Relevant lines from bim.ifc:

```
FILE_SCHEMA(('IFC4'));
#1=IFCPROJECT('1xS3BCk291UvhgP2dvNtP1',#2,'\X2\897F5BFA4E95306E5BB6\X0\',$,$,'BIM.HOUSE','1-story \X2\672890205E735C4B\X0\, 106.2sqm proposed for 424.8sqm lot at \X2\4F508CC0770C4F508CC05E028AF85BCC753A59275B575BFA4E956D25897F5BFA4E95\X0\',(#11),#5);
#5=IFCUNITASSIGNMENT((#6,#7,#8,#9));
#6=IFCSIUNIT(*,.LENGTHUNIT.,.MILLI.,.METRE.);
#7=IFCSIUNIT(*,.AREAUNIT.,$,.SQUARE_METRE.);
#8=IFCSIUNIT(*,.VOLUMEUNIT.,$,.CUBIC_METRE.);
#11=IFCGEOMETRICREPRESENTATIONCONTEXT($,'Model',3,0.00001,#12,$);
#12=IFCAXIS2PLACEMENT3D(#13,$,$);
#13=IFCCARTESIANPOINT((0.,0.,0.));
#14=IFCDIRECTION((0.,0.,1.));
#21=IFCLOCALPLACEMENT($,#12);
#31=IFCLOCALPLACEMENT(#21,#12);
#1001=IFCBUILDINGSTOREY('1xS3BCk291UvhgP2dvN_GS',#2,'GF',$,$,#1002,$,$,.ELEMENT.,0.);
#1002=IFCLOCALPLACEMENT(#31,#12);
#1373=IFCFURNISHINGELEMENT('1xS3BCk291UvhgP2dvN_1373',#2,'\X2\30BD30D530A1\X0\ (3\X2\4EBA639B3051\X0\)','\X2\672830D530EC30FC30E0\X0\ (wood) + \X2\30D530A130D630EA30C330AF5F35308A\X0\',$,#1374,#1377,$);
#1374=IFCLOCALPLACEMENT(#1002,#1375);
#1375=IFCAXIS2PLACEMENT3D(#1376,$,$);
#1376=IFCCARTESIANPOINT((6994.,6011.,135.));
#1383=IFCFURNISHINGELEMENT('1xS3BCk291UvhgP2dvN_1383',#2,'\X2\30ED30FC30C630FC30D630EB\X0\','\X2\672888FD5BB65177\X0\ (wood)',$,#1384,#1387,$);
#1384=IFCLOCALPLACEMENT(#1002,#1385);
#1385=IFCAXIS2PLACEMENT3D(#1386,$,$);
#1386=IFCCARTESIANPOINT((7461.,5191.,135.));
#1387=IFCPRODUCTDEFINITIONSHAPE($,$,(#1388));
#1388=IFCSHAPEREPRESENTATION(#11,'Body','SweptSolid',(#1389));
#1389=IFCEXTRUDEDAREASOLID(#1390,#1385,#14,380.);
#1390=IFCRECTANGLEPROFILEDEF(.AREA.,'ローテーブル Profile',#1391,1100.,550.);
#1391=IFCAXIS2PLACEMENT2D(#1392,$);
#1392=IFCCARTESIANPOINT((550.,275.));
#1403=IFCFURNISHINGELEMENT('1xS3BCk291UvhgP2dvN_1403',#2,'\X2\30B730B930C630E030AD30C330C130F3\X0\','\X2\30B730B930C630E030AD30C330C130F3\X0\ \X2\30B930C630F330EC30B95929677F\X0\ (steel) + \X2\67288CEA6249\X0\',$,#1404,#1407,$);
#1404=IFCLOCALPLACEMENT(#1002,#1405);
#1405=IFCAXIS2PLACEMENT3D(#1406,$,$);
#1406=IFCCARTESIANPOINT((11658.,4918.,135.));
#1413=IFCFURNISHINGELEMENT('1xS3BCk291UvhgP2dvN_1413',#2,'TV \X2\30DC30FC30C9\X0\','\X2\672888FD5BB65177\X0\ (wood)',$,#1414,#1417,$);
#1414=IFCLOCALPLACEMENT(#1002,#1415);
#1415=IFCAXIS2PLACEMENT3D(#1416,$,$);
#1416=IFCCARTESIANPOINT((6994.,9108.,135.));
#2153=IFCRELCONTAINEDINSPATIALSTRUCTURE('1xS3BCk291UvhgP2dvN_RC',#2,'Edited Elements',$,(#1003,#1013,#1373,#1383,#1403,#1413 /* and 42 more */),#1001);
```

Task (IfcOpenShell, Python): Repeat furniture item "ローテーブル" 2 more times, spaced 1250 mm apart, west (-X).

```python
import numpy as np
import ifcopenshell
import ifcopenshell.api.geometry
import ifcopenshell.api.root
import ifcopenshell.util.element
import ifcopenshell.util.placement
import ifcopenshell.util.unit

model = ifcopenshell.open("bim.ifc")
unit_scale = ifcopenshell.util.unit.calculate_unit_scale(model)


def reuse_history(source, copy):
    """copy_class also copies each property set's owner history, people and application; keep the originals."""
    for rel in copy.IsDefinedBy:
        if rel.is_a("IfcRelDefinesByProperties") and (history := rel.RelatingPropertyDefinition.OwnerHistory):
            rel.RelatingPropertyDefinition.OwnerHistory = source.OwnerHistory
            ifcopenshell.util.element.remove_deep2(model, history)


source = model.by_guid("1xS3BCk291UvhgP2dvN_1383")
base = ifcopenshell.util.placement.get_local_placement(source.ObjectPlacement)
step = np.array([-1.0, 0.0, 0.0]) * 1.25 / unit_scale

for i in range(1, 3):
    copy = ifcopenshell.api.root.copy_class(model, product=source)
    copy.Representation = ifcopenshell.util.element.copy_deep(
        model, source.Representation, exclude=["IfcGeometricRepresentationContext", "IfcRepresentationMap"]
    )
    reuse_history(source, copy)
    matrix = base.copy()
    matrix[:3, 3] += i * step
    print("added at", matrix[:3, 3].round(3) + 0.0)
    ifcopenshell.api.geometry.edit_object_placement(model, product=copy, matrix=matrix, is_si=False)

model.write("bim-out.ifc")
```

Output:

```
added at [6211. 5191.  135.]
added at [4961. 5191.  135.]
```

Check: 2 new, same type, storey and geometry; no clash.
